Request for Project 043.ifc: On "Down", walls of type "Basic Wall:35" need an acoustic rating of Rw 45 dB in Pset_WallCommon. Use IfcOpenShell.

First a look at what the model holds.

```python
import ifcopenshell
import ifcopenshell.util.element

model = ifcopenshell.open("Project 043.ifc")
print(model.schema)
storey = next(s for s in model.by_type("IfcBuildingStorey") if s.Name == "Down")
walls = [e for e in ifcopenshell.util.element.get_decomposition(storey) if e.is_a("IfcWall")]
seen = {}
for e in walls:
    element_type = ifcopenshell.util.element.get_type(e)
    key = (element_type.Name if element_type != e and element_type else None, ifcopenshell.util.element.get_pset(e, "Pset_WallCommon", "AcousticRating"))
    seen[key] = seen.get(key, 0) + 1
for (name, value), count in sorted(seen.items(), key=str):
    print(count, "x", name, "|", value)
```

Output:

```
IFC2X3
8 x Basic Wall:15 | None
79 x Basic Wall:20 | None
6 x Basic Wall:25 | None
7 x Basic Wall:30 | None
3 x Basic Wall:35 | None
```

```python
import ifcopenshell
import ifcopenshell.api.pset
import ifcopenshell.util.element

model = ifcopenshell.open("Project 043.ifc")

storey = next(s for s in model.by_type("IfcBuildingStorey") if s.Name == "Down")
walls = [e for e in ifcopenshell.util.element.get_decomposition(storey) if e.is_a("IfcWall")]

count = 0
for e in walls:
    element_type = ifcopenshell.util.element.get_type(e)
    if element_type in (None, e) or element_type.Name != "Basic Wall:35":
        continue
    # add_pset returns the element's existing set when there is one.
    pset = ifcopenshell.api.pset.add_pset(model, product=e, name="Pset_WallCommon")
    ifcopenshell.api.pset.edit_pset(model, pset=pset, properties={"AcousticRating": "Rw 45 dB"})
    count += 1

print(count, "walls updated")

model.write("Project 043_rev.ifc")
```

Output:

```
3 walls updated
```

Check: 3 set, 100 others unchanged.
